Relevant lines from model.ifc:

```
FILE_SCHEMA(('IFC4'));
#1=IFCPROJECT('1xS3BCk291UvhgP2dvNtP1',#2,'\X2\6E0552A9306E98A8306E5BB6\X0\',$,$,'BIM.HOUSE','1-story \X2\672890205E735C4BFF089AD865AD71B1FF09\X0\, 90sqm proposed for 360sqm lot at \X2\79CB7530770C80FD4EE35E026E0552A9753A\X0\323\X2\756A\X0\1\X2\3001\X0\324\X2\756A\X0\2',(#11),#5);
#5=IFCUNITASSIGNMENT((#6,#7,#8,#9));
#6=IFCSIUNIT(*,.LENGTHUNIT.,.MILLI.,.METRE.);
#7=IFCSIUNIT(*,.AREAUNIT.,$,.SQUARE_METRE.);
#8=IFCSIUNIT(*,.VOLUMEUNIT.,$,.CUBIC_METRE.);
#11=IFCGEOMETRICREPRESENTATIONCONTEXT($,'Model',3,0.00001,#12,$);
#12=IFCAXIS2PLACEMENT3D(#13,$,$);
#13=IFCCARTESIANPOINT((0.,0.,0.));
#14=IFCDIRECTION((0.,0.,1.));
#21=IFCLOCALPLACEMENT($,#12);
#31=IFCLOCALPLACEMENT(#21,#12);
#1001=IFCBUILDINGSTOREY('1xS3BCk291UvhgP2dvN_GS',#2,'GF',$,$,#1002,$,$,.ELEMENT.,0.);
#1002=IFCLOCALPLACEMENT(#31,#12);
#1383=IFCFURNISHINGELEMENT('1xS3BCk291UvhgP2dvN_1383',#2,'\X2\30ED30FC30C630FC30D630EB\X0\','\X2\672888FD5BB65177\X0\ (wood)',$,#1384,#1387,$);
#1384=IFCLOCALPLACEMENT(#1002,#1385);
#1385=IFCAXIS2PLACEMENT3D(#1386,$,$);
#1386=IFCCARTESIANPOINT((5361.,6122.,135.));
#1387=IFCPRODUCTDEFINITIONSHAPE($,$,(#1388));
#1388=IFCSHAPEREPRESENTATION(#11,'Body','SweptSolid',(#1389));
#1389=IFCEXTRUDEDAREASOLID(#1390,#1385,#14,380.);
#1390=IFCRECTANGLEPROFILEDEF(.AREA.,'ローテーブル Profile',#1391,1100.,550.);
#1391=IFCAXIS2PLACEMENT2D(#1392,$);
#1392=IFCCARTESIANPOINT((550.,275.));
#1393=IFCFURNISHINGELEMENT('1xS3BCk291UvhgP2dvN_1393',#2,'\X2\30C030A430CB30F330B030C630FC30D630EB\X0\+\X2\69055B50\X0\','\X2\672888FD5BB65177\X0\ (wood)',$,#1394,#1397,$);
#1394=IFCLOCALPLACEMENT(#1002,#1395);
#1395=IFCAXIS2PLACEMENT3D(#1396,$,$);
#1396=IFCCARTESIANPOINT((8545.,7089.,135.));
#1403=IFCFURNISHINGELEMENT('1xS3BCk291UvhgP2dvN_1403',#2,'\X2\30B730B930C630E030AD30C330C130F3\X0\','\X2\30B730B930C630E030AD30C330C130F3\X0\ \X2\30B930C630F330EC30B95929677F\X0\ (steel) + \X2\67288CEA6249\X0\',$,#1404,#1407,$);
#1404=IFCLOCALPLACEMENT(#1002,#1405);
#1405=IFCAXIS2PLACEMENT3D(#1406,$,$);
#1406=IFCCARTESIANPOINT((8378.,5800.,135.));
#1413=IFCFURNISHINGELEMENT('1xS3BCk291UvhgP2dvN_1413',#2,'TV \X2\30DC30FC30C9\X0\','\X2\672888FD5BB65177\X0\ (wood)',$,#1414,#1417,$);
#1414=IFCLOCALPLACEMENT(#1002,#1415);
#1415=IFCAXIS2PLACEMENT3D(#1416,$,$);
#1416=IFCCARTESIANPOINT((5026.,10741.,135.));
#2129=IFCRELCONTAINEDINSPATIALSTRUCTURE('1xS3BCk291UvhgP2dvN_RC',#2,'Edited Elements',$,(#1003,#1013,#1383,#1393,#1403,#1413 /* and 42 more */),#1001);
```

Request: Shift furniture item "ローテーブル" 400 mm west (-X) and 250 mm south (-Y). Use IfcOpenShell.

```python
import ifcopenshell
import ifcopenshell.api.geometry
import ifcopenshell.util.placement

model = ifcopenshell.open("model.ifc")

item = model.by_guid("1xS3BCk291UvhgP2dvN_1383")
matrix = ifcopenshell.util.placement.get_local_placement(item.ObjectPlacement)
matrix[0, 3] -= 400.0
matrix[1, 3] -= 250.0
ifcopenshell.api.geometry.edit_object_placement(model, product=item, matrix=matrix, is_si=False)

print(ifcopenshell.util.placement.get_local_placement(item.ObjectPlacement).round(3) + 0.0)

model.write("model_edited.ifc")
```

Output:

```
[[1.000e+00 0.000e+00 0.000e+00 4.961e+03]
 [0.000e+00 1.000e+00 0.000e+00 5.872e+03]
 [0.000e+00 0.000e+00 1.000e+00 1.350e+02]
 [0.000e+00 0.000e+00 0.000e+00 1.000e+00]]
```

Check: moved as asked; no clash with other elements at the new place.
